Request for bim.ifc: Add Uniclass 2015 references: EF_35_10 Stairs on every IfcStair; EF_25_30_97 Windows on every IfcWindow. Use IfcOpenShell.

First a look at what the model holds.

```python
import ifcopenshell

model = ifcopenshell.open("bim.ifc")
print(model.schema)
print("classifications:", [c.Name for c in model.by_type("IfcClassification")])
for ifc_class in ("IfcDoor", "IfcRoof", "IfcStair", "IfcWall", "IfcWindow"):
    print(ifc_class, len(model.by_type(ifc_class)))
```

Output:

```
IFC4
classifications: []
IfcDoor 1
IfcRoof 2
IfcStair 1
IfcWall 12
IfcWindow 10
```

```python
import ifcopenshell
import ifcopenshell.api.classification

model = ifcopenshell.open("bim.ifc")

system = ifcopenshell.api.classification.add_classification(model, classification="Uniclass 2015")

codes = {
    "IfcStair": ("EF_35_10", "Stairs"),
    "IfcWindow": ("EF_25_30_97", "Windows"),
}
for ifc_class, (code, name) in codes.items():
    products = model.by_type(ifc_class)
    ifcopenshell.api.classification.add_reference(
        model, products=products, classification=system, identification=code, name=name
    )
    print(code, len(products))

model.write("bim_updated.ifc")
```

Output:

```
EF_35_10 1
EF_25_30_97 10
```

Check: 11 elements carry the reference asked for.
